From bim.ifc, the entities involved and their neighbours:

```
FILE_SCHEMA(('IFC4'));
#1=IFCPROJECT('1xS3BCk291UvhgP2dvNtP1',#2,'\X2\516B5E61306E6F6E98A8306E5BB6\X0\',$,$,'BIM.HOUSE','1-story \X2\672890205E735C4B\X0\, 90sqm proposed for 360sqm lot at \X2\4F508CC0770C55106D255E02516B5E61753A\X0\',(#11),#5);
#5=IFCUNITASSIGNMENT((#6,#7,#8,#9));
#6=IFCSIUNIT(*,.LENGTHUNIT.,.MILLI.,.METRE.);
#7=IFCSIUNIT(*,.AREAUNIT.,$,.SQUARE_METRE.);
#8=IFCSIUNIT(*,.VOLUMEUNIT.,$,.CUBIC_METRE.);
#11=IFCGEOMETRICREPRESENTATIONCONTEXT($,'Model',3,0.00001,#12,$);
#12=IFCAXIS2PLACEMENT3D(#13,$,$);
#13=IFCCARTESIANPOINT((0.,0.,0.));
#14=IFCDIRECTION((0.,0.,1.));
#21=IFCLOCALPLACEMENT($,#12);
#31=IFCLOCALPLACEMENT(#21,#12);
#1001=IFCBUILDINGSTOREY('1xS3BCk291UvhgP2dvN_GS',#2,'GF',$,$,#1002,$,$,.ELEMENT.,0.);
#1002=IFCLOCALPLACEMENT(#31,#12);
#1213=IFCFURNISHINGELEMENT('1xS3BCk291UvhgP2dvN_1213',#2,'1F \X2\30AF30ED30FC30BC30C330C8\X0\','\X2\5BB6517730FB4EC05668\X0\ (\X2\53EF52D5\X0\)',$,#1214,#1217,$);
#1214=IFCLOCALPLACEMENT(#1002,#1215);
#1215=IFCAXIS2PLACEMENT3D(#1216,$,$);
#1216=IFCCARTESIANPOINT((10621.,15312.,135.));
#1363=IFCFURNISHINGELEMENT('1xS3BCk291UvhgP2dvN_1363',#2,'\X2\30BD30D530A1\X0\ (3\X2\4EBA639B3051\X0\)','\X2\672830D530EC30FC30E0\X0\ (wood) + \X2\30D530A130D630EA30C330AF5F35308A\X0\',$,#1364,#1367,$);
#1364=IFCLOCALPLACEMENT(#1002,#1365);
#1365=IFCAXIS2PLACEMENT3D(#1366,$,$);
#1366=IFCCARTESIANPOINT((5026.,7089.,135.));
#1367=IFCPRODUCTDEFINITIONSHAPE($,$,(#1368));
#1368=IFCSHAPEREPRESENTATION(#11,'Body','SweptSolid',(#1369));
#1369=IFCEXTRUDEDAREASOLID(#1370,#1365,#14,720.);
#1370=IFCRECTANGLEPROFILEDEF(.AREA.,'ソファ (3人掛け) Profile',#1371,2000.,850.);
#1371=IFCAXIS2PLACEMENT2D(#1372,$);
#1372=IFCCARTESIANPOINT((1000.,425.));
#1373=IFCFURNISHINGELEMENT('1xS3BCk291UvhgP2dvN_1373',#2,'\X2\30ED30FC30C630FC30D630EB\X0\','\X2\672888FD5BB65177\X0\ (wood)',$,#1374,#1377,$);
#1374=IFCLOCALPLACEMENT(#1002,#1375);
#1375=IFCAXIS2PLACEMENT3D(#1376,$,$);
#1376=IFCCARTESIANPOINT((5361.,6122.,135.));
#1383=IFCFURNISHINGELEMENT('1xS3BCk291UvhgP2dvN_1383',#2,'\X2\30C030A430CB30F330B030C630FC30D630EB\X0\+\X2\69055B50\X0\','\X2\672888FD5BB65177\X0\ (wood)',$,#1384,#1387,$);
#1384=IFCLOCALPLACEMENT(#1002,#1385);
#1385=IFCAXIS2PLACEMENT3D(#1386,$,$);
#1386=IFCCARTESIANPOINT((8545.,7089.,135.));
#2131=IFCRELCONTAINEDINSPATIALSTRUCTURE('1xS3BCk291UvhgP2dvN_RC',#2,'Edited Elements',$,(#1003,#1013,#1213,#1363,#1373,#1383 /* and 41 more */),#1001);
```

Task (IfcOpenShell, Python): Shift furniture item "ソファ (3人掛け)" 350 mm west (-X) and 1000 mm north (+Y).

```python
import ifcopenshell
import ifcopenshell.api.geometry
import ifcopenshell.util.placement

model = ifcopenshell.open("bim.ifc")

item = model.by_guid("1xS3BCk291UvhgP2dvN_1363")
matrix = ifcopenshell.util.placement.get_local_placement(item.ObjectPlacement)
matrix[0, 3] -= 350.0
matrix[1, 3] += 1000.0
ifcopenshell.api.geometry.edit_object_placement(model, product=item, matrix=matrix, is_si=False)

print(ifcopenshell.util.placement.get_local_placement(item.ObjectPlacement).round(3) + 0.0)

model.write("bim_edited.ifc")
```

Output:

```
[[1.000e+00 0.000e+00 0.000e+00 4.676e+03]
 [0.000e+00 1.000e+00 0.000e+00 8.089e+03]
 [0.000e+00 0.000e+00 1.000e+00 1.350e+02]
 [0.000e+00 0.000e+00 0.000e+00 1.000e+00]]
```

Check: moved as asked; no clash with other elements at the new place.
